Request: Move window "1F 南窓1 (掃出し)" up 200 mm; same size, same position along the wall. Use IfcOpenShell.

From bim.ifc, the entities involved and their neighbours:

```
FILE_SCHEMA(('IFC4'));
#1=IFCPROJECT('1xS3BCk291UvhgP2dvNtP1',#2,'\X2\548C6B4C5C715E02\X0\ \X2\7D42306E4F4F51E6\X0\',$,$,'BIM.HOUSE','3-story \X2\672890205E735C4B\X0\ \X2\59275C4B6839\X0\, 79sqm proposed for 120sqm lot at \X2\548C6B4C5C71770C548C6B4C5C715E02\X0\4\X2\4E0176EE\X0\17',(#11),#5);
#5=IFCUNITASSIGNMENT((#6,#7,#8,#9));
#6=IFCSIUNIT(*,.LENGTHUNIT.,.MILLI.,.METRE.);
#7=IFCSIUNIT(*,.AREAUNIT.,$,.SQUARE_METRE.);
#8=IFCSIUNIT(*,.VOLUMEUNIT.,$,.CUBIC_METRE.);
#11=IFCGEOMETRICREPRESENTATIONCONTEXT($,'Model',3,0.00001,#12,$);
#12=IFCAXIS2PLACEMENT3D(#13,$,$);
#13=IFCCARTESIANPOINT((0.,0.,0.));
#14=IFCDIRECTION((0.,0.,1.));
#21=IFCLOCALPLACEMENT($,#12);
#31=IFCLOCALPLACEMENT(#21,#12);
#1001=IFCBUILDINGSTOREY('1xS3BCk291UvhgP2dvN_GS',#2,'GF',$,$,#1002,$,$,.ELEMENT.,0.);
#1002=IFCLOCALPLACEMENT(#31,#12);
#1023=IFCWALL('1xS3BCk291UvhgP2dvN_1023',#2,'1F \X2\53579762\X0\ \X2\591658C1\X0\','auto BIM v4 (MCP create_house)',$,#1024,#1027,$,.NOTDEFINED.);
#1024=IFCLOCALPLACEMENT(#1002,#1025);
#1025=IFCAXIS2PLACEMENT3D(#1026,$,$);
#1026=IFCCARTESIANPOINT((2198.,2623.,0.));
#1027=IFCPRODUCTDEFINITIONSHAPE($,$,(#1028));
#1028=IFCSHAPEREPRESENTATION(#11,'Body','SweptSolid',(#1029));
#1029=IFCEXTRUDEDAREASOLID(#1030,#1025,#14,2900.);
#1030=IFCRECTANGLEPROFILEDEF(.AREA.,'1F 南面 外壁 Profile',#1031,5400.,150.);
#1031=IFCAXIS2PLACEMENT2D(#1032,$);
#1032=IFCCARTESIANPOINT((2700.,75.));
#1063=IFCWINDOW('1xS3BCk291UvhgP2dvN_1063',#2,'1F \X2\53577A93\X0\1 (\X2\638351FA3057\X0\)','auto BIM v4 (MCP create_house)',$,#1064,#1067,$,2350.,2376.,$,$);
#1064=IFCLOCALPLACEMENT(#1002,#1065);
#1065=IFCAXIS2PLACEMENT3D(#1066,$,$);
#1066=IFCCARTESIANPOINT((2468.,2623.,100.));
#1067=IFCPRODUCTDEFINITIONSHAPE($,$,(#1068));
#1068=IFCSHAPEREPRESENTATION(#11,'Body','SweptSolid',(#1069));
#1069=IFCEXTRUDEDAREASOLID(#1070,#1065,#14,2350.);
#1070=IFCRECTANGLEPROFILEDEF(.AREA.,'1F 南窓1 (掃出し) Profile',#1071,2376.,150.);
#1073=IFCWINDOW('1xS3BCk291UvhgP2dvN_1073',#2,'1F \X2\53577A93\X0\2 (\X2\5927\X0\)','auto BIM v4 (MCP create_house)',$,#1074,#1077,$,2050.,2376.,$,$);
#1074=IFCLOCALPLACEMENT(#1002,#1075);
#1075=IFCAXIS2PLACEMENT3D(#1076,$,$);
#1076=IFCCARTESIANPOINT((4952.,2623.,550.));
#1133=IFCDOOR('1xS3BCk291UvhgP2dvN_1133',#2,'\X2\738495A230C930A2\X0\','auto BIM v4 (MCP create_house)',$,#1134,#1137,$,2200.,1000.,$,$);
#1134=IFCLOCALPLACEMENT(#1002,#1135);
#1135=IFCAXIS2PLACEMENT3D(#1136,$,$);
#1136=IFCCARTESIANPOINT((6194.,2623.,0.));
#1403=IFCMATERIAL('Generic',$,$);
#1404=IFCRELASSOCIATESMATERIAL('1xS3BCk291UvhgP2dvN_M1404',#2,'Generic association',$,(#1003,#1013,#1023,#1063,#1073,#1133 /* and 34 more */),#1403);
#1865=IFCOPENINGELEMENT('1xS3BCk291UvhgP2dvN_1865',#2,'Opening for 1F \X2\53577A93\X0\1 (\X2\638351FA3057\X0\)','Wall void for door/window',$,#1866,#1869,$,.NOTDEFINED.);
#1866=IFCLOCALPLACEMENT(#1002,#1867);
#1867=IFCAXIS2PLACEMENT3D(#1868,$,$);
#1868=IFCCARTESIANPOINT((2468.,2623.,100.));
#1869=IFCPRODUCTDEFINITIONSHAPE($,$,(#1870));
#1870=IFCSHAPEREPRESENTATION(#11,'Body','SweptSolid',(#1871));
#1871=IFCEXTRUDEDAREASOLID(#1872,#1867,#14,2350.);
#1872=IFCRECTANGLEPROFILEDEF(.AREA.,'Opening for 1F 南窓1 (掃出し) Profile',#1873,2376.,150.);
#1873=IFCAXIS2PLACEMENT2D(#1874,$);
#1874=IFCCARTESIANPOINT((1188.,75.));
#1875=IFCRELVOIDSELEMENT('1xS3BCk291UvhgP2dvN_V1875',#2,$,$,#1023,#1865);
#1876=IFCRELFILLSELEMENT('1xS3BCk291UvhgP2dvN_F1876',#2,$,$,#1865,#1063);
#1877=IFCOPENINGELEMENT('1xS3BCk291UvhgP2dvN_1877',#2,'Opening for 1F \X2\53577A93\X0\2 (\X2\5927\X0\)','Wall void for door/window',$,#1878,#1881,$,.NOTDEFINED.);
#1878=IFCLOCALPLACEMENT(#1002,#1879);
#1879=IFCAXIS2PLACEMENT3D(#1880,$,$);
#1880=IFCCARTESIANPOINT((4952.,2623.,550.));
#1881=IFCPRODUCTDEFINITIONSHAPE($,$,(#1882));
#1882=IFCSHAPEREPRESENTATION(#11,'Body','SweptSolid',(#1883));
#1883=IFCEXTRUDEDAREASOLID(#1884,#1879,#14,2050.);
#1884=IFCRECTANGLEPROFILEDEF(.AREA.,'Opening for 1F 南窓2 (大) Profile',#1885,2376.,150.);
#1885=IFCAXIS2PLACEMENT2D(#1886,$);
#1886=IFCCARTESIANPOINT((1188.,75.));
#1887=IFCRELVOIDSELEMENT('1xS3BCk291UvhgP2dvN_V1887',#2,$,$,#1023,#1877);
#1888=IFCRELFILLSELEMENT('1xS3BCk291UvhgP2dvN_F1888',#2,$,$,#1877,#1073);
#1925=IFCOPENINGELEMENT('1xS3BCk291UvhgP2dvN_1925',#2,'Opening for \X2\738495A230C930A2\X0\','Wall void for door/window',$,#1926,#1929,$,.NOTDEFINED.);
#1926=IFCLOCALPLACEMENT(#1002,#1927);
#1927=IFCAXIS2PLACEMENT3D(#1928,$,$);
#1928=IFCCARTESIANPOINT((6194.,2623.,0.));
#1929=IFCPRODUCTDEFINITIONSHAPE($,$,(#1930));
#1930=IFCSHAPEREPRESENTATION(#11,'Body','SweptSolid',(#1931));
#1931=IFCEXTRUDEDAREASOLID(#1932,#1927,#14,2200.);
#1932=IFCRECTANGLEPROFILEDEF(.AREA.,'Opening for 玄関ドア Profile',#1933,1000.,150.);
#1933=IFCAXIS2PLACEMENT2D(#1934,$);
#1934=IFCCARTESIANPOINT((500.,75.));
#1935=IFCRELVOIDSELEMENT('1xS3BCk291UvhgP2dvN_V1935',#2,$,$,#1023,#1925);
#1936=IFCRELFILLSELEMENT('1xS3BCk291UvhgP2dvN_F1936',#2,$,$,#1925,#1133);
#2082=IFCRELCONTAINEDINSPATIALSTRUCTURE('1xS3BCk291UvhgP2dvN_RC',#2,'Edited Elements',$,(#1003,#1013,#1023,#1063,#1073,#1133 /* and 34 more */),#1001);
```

```python
import numpy as np
import ifcopenshell
import ifcopenshell.api.geometry
import ifcopenshell.util.placement
import ifcopenshell.util.unit

model = ifcopenshell.open("bim.ifc")
unit_scale = ifcopenshell.util.unit.calculate_unit_scale(model)

window = model.by_guid("1xS3BCk291UvhgP2dvN_1063")
opening = window.FillsVoids[0].RelatingOpeningElement
dz = 0.2 / unit_scale

shift = np.array([0.0, 0.0, dz])
# The window is not placed relative to its opening, so move both.
for product in (opening, window):
    matrix = ifcopenshell.util.placement.get_local_placement(product.ObjectPlacement)
    matrix[:3, 3] += shift
    ifcopenshell.api.geometry.edit_object_placement(model, product=product, matrix=matrix, is_si=False)

print(f"moved by {dz * unit_scale:+.3f} m")

model.write("bim-out.ifc")
```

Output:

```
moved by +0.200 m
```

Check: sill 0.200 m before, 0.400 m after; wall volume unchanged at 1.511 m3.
